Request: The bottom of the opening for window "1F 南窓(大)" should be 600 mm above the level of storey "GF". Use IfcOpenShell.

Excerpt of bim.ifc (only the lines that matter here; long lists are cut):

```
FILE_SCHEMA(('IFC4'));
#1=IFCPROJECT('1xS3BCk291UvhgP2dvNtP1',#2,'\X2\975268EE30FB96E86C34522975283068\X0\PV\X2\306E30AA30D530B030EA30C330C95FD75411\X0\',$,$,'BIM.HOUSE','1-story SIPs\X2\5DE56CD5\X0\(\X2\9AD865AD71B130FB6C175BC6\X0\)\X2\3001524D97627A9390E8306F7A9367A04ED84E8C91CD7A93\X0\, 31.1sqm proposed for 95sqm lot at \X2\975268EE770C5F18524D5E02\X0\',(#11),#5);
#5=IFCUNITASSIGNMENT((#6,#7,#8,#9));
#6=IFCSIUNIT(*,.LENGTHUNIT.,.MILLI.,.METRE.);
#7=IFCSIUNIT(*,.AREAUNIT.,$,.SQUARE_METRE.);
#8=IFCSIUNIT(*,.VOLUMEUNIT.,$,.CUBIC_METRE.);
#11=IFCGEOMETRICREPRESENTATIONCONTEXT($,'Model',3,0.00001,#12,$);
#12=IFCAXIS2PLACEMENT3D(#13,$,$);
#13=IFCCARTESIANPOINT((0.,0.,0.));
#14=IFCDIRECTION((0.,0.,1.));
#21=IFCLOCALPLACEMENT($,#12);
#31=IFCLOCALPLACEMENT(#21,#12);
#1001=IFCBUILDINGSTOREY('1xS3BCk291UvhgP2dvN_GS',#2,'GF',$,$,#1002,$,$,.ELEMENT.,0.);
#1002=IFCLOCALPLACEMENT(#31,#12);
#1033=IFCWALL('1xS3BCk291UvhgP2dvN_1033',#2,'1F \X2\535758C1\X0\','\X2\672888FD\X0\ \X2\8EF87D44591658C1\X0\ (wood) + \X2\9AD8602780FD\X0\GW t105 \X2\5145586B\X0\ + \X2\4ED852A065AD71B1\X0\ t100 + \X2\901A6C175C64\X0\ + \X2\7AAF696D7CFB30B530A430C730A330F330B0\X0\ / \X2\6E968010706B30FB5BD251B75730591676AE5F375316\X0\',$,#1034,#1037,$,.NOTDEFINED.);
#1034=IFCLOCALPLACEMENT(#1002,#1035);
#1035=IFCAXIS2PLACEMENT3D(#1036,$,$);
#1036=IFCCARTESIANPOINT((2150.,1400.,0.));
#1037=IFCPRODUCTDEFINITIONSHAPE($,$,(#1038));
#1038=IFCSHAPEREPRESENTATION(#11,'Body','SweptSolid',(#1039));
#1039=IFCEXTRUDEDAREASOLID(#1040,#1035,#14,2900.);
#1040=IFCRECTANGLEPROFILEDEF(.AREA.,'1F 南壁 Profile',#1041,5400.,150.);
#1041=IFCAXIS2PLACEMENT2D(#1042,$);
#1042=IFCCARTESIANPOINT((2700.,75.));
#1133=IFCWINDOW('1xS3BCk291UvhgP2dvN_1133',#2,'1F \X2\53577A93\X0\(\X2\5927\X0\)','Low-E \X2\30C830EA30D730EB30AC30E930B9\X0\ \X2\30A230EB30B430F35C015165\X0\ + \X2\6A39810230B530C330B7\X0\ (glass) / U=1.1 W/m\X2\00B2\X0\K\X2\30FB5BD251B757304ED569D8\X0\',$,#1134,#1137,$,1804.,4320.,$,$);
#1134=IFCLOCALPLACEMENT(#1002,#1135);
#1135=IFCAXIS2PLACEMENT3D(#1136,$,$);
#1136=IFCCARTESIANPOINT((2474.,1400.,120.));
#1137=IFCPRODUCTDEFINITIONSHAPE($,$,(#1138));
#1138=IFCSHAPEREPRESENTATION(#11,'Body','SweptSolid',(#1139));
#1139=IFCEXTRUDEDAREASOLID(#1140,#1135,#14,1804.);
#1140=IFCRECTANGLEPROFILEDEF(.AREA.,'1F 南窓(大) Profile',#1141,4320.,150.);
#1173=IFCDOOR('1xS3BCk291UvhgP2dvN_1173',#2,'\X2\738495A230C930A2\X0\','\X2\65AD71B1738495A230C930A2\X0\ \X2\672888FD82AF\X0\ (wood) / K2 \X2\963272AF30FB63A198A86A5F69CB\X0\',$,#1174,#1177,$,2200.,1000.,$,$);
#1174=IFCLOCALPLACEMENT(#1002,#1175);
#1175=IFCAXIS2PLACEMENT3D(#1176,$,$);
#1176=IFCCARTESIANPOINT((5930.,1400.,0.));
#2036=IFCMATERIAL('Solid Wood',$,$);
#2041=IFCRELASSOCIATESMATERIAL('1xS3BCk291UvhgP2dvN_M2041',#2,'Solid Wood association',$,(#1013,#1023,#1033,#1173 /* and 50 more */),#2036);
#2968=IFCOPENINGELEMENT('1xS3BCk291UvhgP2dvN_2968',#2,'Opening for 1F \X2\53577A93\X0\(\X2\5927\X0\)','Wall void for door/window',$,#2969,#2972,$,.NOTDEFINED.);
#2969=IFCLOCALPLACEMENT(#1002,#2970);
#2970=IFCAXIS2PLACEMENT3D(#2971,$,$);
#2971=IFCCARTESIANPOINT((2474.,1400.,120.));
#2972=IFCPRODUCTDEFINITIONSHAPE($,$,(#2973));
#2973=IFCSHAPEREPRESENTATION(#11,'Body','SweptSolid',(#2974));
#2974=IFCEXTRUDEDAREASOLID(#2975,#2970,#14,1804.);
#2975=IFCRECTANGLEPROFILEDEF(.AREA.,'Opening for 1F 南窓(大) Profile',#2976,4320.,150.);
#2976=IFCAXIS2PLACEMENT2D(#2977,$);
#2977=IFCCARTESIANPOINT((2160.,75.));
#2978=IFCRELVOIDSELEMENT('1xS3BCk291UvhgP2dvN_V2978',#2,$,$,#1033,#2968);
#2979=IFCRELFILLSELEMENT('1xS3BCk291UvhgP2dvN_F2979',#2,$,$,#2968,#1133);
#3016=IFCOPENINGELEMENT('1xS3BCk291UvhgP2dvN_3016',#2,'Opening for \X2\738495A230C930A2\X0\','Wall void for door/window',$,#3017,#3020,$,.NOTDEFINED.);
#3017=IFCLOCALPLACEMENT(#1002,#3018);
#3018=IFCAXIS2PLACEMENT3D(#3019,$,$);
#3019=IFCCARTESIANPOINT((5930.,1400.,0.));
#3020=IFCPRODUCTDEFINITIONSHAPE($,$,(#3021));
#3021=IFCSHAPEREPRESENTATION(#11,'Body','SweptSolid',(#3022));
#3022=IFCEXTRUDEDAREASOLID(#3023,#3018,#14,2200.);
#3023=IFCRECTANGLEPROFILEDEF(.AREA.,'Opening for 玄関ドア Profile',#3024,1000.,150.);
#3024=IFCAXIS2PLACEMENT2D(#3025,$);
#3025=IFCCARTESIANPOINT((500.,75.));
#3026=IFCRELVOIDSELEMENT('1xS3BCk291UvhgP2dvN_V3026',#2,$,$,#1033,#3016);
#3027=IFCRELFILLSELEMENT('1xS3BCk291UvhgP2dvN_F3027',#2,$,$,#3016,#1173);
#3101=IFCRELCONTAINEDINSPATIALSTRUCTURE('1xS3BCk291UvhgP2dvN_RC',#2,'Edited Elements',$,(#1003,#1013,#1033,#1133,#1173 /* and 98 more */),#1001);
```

```python
import numpy as np
import ifcopenshell
import ifcopenshell.api.geometry
import ifcopenshell.geom
import ifcopenshell.util.element
import ifcopenshell.util.placement
import ifcopenshell.util.shape
import ifcopenshell.util.unit

model = ifcopenshell.open("bim.ifc")
unit_scale = ifcopenshell.util.unit.calculate_unit_scale(model)

window = model.by_guid("1xS3BCk291UvhgP2dvN_1133")
opening = window.FillsVoids[0].RelatingOpeningElement
storey = ifcopenshell.util.element.get_container(window, ifc_class="IfcBuildingStorey")
level = ifcopenshell.util.placement.get_local_placement(storey.ObjectPlacement)[2, 3]

# The opening's origin need not be at the sill, so measure its lowest point.
shape = ifcopenshell.geom.create_shape(ifcopenshell.geom.settings(), opening)
bottom = ifcopenshell.util.shape.get_shape_bottom_elevation(shape, shape.geometry) / unit_scale
dz = level + 0.6 / unit_scale - bottom

shift = np.array([0.0, 0.0, dz])
# The window is not placed relative to its opening, so move both.
for product in (opening, window):
    matrix = ifcopenshell.util.placement.get_local_placement(product.ObjectPlacement)
    matrix[:3, 3] += shift
    ifcopenshell.api.geometry.edit_object_placement(model, product=product, matrix=matrix, is_si=False)

print(f"moved by {dz * unit_scale:+.3f} m")

model.write("bim_updated.ifc")
```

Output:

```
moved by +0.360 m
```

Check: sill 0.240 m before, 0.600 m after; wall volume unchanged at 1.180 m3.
